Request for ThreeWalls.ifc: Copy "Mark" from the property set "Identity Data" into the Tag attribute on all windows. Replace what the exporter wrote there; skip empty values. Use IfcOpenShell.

First a look at what the model holds.

```python
import ifcopenshell
import ifcopenshell.util.element

model = ifcopenshell.open("ThreeWalls.ifc")
print(model.schema)
windows = model.by_type("IfcWindow")
print(len(windows), "windows")
for e in windows[:8]:
    source = ifcopenshell.util.element.get_pset(e, "Identity Data", "Mark")
    target = e.Tag
    print(e.id(), repr(source), repr(target), sep=" | ")
```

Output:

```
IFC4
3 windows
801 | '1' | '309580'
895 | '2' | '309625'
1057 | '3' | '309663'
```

```python
import ifcopenshell
import ifcopenshell.util.element

model = ifcopenshell.open("ThreeWalls.ifc")

count = 0
for e in model.by_type("IfcWindow"):
    value = ifcopenshell.util.element.get_pset(e, "Identity Data", "Mark")
    current = e.Tag
    if not value or not value.strip() or current == value:
        continue
    e.Tag = value
    count += 1

print(count, "windows updated")

model.write("ThreeWalls_updated.ifc")
```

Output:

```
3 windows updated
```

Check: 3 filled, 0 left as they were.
